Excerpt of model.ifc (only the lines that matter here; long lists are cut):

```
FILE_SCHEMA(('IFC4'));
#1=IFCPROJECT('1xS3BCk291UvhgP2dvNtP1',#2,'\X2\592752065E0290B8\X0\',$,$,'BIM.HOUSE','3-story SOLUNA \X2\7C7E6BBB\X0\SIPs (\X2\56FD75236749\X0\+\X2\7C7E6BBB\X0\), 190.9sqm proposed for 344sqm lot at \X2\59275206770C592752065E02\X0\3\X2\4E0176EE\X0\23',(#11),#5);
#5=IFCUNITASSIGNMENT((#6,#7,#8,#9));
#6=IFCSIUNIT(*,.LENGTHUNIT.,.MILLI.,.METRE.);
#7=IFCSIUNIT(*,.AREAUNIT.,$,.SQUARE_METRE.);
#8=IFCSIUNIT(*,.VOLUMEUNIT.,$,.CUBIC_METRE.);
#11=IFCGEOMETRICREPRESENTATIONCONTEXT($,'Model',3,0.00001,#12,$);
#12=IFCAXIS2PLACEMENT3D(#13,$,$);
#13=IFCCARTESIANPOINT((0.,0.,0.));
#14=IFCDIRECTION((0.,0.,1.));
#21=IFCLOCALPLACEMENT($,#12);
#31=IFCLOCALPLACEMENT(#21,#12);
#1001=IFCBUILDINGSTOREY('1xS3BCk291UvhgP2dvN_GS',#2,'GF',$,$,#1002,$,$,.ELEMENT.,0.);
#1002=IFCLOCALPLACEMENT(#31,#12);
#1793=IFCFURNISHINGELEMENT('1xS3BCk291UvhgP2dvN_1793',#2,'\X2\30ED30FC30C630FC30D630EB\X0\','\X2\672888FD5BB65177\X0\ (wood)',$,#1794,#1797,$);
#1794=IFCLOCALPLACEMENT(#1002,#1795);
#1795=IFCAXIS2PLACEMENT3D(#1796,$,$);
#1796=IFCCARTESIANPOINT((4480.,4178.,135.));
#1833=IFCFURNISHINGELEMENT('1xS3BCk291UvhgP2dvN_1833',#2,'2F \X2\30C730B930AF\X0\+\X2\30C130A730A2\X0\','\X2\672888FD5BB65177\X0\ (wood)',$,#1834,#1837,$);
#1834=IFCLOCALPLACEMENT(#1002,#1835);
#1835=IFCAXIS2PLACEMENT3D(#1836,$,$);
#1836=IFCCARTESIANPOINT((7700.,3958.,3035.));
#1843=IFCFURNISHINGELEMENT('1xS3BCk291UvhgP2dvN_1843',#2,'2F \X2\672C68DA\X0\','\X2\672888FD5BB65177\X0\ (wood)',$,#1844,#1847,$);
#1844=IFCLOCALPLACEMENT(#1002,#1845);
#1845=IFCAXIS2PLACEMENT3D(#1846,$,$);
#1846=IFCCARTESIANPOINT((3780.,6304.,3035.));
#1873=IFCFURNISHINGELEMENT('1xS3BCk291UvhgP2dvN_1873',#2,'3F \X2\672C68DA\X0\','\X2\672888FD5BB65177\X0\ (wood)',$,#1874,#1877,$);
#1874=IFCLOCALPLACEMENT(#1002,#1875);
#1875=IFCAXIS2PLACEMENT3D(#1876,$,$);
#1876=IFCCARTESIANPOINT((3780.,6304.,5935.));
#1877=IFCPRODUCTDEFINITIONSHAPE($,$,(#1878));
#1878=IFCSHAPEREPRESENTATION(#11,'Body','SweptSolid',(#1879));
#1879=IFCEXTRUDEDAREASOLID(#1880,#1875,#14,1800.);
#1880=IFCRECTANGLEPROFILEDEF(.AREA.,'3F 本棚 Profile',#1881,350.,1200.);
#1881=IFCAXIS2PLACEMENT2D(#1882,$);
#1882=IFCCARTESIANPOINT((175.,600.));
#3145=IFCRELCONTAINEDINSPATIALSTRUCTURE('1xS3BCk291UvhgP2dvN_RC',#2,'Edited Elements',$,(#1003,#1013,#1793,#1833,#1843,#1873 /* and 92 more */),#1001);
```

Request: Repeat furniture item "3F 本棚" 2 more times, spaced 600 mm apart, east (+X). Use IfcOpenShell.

```python
import numpy as np
import ifcopenshell
import ifcopenshell.api.geometry
import ifcopenshell.api.root
import ifcopenshell.util.element
import ifcopenshell.util.placement
import ifcopenshell.util.unit

model = ifcopenshell.open("model.ifc")
unit_scale = ifcopenshell.util.unit.calculate_unit_scale(model)


def reuse_history(source, copy):
    """copy_class also copies each property set's owner history, people and application; keep the originals."""
    for rel in copy.IsDefinedBy:
        if rel.is_a("IfcRelDefinesByProperties") and (history := rel.RelatingPropertyDefinition.OwnerHistory):
            rel.RelatingPropertyDefinition.OwnerHistory = source.OwnerHistory
            ifcopenshell.util.element.remove_deep2(model, history)


source = model.by_guid("1xS3BCk291UvhgP2dvN_1873")
base = ifcopenshell.util.placement.get_local_placement(source.ObjectPlacement)
step = np.array([1.0, 0.0, 0.0]) * 0.6 / unit_scale

for i in range(1, 3):
    copy = ifcopenshell.api.root.copy_class(model, product=source)
    copy.Representation = ifcopenshell.util.element.copy_deep(
        model, source.Representation, exclude=["IfcGeometricRepresentationContext", "IfcRepresentationMap"]
    )
    reuse_history(source, copy)
    matrix = base.copy()
    matrix[:3, 3] += i * step
    print("added at", matrix[:3, 3].round(3) + 0.0)
    ifcopenshell.api.geometry.edit_object_placement(model, product=copy, matrix=matrix, is_si=False)

model.write("model_edited.ifc")
```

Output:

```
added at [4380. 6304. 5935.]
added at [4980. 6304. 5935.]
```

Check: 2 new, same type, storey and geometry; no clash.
